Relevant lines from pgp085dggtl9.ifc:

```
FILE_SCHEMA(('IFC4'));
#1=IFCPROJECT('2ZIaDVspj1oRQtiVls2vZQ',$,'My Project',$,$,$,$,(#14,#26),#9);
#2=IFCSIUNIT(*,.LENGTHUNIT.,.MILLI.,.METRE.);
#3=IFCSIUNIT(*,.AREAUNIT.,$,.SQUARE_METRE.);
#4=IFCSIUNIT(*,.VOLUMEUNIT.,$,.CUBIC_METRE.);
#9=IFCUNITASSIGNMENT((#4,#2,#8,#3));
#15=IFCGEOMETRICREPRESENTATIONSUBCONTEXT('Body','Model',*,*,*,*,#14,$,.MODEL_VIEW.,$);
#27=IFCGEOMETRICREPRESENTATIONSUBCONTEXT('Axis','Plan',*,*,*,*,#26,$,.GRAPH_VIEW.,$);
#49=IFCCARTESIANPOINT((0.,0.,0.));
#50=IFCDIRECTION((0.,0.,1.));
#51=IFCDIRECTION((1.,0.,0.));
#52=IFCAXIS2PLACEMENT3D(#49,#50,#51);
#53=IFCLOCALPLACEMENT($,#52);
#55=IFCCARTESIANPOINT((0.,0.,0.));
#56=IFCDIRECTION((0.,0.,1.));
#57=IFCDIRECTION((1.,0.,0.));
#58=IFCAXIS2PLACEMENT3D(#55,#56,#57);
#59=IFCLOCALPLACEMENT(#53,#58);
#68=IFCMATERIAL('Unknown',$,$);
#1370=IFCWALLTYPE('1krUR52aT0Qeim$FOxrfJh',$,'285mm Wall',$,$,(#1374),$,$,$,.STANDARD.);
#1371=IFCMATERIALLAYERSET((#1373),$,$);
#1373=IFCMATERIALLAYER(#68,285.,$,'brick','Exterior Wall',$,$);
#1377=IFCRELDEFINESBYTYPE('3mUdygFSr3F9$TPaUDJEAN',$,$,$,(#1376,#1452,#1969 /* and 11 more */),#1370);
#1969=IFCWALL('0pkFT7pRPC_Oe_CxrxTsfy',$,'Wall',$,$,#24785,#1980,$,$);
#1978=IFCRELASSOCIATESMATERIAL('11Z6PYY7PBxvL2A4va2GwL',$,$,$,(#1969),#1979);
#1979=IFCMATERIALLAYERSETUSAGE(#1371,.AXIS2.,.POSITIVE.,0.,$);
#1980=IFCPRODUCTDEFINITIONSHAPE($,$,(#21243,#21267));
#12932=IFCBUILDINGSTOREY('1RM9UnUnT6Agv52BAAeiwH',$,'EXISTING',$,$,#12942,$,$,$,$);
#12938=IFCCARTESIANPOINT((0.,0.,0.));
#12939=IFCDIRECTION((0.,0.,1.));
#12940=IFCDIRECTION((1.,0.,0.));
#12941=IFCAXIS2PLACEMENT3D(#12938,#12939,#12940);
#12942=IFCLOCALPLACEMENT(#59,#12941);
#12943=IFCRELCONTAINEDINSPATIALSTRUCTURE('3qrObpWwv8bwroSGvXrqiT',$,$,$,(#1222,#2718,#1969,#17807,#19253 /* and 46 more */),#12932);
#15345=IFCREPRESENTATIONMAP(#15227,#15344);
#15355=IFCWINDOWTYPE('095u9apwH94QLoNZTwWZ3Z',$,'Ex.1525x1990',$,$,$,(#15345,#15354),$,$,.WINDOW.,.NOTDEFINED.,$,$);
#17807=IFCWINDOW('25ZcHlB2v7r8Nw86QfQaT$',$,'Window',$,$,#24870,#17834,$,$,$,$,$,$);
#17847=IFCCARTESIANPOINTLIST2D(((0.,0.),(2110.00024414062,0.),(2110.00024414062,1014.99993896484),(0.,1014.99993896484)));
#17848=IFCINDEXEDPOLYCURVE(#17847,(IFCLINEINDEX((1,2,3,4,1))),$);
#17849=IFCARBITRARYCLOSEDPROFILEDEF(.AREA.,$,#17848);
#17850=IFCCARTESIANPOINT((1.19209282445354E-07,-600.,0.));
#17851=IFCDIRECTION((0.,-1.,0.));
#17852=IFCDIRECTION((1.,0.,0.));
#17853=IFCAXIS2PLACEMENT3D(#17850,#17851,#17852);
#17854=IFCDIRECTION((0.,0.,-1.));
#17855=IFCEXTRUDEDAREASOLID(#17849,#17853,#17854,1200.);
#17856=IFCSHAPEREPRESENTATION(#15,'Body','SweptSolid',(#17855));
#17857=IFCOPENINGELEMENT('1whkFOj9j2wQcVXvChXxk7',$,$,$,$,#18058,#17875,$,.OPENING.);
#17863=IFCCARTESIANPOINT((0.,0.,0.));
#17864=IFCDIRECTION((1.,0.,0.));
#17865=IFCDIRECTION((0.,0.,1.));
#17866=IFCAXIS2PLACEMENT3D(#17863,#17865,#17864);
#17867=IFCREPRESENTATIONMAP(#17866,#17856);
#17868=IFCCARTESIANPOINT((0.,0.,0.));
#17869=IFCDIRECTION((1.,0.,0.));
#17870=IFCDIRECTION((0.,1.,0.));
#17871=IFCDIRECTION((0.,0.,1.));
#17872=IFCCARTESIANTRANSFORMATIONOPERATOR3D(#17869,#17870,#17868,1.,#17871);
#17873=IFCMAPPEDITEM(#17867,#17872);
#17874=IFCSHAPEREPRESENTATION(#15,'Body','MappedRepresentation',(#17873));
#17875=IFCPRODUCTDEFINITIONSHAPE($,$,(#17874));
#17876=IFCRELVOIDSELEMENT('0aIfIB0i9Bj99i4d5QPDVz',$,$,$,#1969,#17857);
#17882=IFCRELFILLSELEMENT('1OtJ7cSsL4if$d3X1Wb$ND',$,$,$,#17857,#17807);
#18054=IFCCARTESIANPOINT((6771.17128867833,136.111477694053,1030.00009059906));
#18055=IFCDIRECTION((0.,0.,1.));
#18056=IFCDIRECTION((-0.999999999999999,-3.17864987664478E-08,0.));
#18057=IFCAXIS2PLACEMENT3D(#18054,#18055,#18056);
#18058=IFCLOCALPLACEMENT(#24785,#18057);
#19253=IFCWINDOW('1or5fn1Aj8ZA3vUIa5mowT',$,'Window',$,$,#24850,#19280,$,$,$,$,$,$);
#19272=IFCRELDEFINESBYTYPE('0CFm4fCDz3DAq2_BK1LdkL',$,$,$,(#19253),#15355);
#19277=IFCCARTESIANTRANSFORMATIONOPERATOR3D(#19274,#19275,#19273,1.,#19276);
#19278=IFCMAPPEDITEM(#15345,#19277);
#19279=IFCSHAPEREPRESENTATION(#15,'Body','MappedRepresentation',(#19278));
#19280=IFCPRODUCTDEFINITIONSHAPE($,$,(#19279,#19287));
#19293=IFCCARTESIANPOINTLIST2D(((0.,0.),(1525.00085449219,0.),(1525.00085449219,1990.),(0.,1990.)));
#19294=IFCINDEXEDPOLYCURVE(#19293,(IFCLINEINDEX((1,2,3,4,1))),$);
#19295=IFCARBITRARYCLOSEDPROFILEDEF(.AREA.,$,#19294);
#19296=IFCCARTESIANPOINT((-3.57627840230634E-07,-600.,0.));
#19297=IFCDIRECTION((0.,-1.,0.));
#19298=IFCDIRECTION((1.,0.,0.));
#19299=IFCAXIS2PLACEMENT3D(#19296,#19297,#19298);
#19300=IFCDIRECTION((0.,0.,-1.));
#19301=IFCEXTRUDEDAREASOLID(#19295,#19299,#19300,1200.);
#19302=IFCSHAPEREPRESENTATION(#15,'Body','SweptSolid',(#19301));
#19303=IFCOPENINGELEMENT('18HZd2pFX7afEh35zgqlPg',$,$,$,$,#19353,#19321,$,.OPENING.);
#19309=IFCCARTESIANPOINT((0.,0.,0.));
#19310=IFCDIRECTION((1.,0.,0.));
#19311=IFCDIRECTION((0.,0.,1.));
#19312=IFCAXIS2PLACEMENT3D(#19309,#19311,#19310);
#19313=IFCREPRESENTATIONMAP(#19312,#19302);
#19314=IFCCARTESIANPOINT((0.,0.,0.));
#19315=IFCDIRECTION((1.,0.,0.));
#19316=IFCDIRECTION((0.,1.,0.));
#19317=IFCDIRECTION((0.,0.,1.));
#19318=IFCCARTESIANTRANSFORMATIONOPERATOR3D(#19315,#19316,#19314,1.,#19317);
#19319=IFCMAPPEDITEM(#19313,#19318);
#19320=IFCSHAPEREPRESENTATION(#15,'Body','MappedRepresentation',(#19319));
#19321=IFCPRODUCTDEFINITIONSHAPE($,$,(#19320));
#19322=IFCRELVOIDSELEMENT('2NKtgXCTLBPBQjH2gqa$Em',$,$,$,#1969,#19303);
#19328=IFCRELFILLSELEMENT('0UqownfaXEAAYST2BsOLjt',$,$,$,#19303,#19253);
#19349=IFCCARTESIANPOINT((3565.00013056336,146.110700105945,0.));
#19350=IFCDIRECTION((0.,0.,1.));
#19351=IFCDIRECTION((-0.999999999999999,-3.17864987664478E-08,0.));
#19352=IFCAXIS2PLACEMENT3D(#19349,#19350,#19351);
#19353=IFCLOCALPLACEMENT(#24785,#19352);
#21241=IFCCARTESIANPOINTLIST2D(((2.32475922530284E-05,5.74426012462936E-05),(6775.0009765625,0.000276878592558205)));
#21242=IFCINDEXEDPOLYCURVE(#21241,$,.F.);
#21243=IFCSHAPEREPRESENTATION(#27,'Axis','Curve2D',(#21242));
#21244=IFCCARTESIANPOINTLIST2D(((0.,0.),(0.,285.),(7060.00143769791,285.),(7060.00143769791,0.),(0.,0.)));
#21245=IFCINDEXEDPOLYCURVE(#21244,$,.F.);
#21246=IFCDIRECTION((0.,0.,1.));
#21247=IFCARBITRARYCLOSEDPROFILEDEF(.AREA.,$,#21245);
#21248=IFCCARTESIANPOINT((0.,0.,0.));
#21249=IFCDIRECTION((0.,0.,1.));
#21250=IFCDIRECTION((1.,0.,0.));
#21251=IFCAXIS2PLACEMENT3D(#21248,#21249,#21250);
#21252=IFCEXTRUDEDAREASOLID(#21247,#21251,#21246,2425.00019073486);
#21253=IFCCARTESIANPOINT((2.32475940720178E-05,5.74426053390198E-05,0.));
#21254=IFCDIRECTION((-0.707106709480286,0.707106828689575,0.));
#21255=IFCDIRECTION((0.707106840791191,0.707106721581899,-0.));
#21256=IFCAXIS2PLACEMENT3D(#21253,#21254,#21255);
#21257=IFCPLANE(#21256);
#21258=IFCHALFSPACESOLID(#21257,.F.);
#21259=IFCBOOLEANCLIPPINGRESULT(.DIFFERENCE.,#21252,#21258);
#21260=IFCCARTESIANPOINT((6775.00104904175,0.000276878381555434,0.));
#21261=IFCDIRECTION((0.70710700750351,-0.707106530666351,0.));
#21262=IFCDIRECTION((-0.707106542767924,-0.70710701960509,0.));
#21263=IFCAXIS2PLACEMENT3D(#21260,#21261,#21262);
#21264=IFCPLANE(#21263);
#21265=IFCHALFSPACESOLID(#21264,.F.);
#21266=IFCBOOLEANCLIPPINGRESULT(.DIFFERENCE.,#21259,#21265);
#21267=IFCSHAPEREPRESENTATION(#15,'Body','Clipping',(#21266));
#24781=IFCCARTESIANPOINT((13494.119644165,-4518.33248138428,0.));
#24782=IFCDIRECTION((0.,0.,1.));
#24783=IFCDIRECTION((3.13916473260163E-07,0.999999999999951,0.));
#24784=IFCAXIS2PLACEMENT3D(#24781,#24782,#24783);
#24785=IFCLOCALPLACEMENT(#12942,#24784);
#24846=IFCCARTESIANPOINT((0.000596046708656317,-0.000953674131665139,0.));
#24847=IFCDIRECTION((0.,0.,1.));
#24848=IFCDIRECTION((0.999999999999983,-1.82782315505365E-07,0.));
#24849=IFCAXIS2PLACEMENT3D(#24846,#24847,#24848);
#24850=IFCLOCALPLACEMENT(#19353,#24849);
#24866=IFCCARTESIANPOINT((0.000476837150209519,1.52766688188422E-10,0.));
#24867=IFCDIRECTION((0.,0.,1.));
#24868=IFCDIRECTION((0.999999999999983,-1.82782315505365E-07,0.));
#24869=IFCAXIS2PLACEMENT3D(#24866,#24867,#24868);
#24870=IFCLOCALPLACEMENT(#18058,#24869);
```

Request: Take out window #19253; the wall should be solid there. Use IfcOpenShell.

```python
import ifcopenshell
import ifcopenshell.api.feature
import ifcopenshell.api.root
import ifcopenshell.geom
import ifcopenshell.util.shape

model = ifcopenshell.open("pgp085dggtl9.ifc")
settings = ifcopenshell.geom.settings()


def volume(element):
    """Net volume in cubic metres, openings subtracted."""
    shape = ifcopenshell.geom.create_shape(settings, element)
    return ifcopenshell.util.shape.get_volume(shape.geometry)


window = model.by_id(19253)
opening = window.FillsVoids[0].RelatingOpeningElement
wall = opening.VoidsElements[0].RelatingBuildingElement
before = volume(wall)

ifcopenshell.api.root.remove_product(model, product=window)
ifcopenshell.api.feature.remove_feature(model, feature=opening)

after = volume(wall)

print(f"wall volume {before:.3f} -> {after:.3f} m3")

model.write("pgp085dggtl9_rev.ifc")
```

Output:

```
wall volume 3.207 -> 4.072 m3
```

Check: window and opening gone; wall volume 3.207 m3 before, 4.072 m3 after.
